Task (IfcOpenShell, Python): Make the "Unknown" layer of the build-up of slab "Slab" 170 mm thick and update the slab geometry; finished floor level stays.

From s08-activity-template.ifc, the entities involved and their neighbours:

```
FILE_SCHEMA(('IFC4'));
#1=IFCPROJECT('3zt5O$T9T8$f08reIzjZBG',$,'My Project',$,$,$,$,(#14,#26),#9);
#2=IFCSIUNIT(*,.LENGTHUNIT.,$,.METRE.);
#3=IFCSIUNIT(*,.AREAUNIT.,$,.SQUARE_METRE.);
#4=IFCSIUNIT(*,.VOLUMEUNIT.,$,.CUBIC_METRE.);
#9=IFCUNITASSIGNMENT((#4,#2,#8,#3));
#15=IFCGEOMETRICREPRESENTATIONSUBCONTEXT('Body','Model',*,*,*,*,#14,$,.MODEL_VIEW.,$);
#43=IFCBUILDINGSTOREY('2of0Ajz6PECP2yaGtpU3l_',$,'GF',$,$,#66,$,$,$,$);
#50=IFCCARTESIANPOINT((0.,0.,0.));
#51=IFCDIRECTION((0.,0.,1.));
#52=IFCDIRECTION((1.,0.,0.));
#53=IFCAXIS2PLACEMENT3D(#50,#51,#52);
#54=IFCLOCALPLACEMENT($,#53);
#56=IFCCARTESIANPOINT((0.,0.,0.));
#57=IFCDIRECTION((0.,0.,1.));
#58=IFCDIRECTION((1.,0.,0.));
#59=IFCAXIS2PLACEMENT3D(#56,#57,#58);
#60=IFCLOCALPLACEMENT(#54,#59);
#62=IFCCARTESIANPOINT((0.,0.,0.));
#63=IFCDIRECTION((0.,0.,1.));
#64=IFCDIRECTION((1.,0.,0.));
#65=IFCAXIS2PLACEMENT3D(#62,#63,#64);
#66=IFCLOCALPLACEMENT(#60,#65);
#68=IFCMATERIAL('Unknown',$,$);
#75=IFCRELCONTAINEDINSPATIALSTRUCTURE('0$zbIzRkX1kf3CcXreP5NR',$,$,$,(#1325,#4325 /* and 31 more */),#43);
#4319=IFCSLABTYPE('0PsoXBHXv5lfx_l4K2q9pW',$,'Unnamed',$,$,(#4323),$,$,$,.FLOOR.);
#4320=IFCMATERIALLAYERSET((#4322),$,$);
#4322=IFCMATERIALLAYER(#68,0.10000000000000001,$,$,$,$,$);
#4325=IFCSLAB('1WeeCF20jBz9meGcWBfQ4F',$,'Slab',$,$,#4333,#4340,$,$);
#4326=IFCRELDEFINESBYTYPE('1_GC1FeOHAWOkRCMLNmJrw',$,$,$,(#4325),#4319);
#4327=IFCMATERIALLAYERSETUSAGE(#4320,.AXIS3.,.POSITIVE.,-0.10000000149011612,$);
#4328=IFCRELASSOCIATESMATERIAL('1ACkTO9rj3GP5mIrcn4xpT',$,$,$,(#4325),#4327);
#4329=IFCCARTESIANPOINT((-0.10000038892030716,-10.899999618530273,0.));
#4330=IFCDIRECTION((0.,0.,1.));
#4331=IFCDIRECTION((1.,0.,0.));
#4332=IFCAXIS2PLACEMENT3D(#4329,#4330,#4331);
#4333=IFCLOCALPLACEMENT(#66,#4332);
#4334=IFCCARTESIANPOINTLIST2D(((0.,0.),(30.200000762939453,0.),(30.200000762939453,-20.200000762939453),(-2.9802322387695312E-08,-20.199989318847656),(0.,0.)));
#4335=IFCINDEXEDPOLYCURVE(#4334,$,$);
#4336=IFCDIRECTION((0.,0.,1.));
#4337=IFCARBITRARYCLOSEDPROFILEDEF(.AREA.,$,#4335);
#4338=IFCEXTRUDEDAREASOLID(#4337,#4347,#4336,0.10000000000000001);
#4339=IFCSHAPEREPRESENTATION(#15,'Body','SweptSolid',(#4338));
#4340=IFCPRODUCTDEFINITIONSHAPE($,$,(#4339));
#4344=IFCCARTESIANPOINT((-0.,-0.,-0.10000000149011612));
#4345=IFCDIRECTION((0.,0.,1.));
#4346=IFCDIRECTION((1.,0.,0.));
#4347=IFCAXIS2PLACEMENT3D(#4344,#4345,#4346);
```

```python
import ifcopenshell
import ifcopenshell.util.element
import ifcopenshell.util.representation
import ifcopenshell.util.unit

model = ifcopenshell.open("s08-activity-template.ifc")
unit_scale = ifcopenshell.util.unit.calculate_unit_scale(model)

layer_set = model.by_id(4320)
layer = next(l for l in layer_set.MaterialLayers if l.Material and l.Material.Name == "Unknown")
change = 0.17 / unit_scale - layer.LayerThickness
layer.LayerThickness += change

# Geometry does not follow the layer set by itself.
slabs = [e for e in ifcopenshell.util.element.get_elements_by_material(model, layer_set) if e.is_a("IfcSlab")]
for slab in sorted(slabs, key=lambda e: e.id()):
    body = ifcopenshell.util.representation.get_representation(slab, "Model", "Body")
    solid = body.Items[0]
    old_depth = solid.Depth
    solid.Depth += change
    # Extruded upwards: lower the start of the extrusion so the top stays.
    x, y, z = solid.Position.Location.Coordinates
    solid.Position.Location = model.createIfcCartesianPoint((x, y, z - change))
    print(slab.id(), f"{old_depth:g} -> {solid.Depth:g}")

# The layers are counted up from the underside, which has moved.
for usage in {ifcopenshell.util.element.get_material(slab) for slab in slabs}:
    usage.OffsetFromReferenceLine -= change

model.write("s08-activity-template_rev.ifc")
```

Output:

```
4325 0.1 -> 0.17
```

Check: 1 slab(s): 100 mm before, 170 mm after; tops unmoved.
